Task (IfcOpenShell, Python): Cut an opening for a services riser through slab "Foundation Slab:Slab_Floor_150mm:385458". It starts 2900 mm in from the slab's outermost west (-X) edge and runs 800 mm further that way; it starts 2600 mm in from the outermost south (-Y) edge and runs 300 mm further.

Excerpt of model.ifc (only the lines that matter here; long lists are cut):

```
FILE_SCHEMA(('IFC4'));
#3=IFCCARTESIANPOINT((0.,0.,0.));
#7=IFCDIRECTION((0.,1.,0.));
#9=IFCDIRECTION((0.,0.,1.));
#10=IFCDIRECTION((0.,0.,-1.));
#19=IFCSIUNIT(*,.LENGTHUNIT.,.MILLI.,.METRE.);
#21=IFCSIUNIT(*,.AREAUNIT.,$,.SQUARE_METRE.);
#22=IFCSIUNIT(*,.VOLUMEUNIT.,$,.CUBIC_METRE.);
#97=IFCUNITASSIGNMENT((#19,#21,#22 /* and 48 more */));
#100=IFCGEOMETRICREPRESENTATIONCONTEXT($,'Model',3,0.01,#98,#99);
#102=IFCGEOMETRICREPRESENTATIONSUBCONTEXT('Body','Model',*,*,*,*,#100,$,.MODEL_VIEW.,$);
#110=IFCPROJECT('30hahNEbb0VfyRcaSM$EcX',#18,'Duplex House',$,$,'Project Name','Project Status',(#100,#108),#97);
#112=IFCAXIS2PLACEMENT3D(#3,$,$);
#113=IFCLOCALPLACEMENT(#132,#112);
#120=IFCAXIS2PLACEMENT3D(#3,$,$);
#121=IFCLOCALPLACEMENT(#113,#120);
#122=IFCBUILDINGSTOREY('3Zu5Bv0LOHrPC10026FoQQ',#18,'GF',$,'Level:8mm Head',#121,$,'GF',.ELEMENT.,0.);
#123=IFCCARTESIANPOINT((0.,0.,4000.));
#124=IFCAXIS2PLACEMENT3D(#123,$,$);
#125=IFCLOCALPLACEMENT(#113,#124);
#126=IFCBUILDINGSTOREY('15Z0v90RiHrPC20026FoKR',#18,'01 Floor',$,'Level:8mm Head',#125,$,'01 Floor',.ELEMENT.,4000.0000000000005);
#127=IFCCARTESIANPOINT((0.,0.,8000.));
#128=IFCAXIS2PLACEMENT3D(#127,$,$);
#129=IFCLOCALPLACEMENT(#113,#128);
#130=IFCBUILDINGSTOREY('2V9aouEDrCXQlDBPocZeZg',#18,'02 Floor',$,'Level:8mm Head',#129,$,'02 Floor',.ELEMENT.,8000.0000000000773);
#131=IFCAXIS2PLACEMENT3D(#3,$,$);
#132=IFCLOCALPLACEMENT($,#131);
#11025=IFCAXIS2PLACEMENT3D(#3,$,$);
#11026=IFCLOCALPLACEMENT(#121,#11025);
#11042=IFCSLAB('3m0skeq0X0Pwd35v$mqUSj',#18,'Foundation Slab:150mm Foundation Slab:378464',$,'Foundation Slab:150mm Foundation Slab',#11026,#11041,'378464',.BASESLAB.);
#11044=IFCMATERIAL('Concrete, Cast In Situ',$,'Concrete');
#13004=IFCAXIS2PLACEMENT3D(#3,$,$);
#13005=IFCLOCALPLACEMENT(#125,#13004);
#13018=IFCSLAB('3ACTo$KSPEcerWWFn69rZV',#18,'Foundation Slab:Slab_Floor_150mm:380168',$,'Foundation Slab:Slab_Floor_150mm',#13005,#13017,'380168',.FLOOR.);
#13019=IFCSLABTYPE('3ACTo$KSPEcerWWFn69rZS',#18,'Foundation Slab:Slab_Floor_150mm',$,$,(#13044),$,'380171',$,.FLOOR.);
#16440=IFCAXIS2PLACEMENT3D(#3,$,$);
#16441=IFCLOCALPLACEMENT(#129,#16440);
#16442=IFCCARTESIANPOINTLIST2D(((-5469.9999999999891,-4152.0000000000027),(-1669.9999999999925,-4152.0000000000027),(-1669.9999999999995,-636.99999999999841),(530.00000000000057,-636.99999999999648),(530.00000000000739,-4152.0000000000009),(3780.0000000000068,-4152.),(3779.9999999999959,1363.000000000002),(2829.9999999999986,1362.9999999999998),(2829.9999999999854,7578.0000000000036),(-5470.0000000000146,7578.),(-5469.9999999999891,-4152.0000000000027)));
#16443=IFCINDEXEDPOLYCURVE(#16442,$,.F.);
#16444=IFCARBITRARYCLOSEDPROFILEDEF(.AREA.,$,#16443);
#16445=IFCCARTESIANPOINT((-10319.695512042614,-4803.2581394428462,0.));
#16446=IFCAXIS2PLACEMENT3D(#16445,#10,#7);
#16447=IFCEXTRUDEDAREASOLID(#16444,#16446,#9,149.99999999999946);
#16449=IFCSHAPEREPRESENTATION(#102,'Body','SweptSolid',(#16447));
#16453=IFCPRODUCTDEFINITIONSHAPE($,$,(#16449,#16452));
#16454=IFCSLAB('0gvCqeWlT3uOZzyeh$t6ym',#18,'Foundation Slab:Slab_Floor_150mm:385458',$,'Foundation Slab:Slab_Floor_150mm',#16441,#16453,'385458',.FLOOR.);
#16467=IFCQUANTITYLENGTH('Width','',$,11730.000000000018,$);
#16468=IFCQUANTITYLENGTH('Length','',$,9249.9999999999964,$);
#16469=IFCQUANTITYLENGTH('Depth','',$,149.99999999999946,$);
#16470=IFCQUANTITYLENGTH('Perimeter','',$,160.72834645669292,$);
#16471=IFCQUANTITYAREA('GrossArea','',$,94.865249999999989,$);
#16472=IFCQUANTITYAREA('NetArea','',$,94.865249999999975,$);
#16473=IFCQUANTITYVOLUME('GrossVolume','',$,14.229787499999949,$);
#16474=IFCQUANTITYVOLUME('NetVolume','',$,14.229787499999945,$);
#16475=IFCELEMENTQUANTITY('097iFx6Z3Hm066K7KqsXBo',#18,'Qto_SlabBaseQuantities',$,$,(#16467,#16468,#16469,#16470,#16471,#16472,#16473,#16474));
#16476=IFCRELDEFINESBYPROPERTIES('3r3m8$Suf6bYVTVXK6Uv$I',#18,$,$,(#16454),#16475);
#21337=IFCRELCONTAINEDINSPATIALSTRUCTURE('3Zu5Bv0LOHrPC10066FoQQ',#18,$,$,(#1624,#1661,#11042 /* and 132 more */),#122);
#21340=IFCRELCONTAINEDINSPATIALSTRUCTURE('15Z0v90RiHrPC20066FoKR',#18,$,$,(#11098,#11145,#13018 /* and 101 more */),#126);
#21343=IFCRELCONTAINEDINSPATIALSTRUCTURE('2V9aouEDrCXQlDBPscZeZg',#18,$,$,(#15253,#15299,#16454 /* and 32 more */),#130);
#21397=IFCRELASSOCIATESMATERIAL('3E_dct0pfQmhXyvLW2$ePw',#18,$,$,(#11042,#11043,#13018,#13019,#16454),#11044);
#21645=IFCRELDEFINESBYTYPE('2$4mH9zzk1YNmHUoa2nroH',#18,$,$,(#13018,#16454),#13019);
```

```python
import numpy as np
import ifcopenshell
import ifcopenshell.api.feature
import ifcopenshell.api.geometry
import ifcopenshell.api.pset
import ifcopenshell.api.root
import ifcopenshell.geom
import ifcopenshell.util.element
import ifcopenshell.util.placement
import ifcopenshell.util.representation
import ifcopenshell.util.shape
import ifcopenshell.util.unit

model = ifcopenshell.open("model.ifc")
unit_scale = ifcopenshell.util.unit.calculate_unit_scale(model)
area_scale = ifcopenshell.util.unit.calculate_unit_scale(model, "AREAUNIT")
volume_scale = ifcopenshell.util.unit.calculate_unit_scale(model, "VOLUMEUNIT")
settings = ifcopenshell.geom.settings()


def volume(element):
    """Net volume in cubic metres, openings subtracted."""
    shape = ifcopenshell.geom.create_shape(settings, element)
    return ifcopenshell.util.shape.get_volume(shape.geometry)


slab = model.by_id(16454)
before = volume(slab)

# Extent in the slab's own axes, in metres. The edges named are its -X and -Y sides.
slab_shape = ifcopenshell.geom.create_shape(settings, slab)
vertices = ifcopenshell.util.shape.get_vertices(slab_shape.geometry)
x_min, y_min, bottom = vertices.min(axis=0)
top = vertices[:, 2].max()

opening = ifcopenshell.api.root.create_entity(model, ifc_class="IfcOpeningElement", name="Services riser opening", predefined_type="OPENING")
context = ifcopenshell.util.representation.get_context(model, "Model", "Body", "MODEL_VIEW")
width, depth = 0.8, 0.3
outline = [(0.0, 0.0), (width, 0.0), (width, depth), (0.0, depth), (0.0, 0.0)]
# Overshoot both faces by 50 mm so the cut is clean.
shape = ifcopenshell.api.geometry.add_slab_representation(
    model, context=context, depth=top - bottom + 0.1, polyline=outline
)
ifcopenshell.api.geometry.assign_representation(model, product=opening, representation=shape)

matrix = ifcopenshell.util.placement.get_local_placement(slab.ObjectPlacement)
matrix[:, 3] = matrix @ np.append(np.array([x_min + 2.9, y_min + 2.6, bottom - 0.05]) / unit_scale, 1.0)
ifcopenshell.api.geometry.edit_object_placement(model, product=opening, matrix=matrix, is_si=False)
ifcopenshell.api.feature.add_feature(model, feature=opening, element=slab)

after = volume(slab)

# Update the slab's stored quantities.
qto = model.by_id(ifcopenshell.util.element.get_pset(slab, "Qto_SlabBaseQuantities", should_inherit=False)["id"])
ifcopenshell.api.pset.edit_qto(model, qto=qto, properties={
    "NetArea": after / (top - bottom) / area_scale,
    "NetVolume": after / volume_scale,
})

print(f"slab volume {before:.3f} -> {after:.3f} m3")

model.write("model_updated.ifc")
```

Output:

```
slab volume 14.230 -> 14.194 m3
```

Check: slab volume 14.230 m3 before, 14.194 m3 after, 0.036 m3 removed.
